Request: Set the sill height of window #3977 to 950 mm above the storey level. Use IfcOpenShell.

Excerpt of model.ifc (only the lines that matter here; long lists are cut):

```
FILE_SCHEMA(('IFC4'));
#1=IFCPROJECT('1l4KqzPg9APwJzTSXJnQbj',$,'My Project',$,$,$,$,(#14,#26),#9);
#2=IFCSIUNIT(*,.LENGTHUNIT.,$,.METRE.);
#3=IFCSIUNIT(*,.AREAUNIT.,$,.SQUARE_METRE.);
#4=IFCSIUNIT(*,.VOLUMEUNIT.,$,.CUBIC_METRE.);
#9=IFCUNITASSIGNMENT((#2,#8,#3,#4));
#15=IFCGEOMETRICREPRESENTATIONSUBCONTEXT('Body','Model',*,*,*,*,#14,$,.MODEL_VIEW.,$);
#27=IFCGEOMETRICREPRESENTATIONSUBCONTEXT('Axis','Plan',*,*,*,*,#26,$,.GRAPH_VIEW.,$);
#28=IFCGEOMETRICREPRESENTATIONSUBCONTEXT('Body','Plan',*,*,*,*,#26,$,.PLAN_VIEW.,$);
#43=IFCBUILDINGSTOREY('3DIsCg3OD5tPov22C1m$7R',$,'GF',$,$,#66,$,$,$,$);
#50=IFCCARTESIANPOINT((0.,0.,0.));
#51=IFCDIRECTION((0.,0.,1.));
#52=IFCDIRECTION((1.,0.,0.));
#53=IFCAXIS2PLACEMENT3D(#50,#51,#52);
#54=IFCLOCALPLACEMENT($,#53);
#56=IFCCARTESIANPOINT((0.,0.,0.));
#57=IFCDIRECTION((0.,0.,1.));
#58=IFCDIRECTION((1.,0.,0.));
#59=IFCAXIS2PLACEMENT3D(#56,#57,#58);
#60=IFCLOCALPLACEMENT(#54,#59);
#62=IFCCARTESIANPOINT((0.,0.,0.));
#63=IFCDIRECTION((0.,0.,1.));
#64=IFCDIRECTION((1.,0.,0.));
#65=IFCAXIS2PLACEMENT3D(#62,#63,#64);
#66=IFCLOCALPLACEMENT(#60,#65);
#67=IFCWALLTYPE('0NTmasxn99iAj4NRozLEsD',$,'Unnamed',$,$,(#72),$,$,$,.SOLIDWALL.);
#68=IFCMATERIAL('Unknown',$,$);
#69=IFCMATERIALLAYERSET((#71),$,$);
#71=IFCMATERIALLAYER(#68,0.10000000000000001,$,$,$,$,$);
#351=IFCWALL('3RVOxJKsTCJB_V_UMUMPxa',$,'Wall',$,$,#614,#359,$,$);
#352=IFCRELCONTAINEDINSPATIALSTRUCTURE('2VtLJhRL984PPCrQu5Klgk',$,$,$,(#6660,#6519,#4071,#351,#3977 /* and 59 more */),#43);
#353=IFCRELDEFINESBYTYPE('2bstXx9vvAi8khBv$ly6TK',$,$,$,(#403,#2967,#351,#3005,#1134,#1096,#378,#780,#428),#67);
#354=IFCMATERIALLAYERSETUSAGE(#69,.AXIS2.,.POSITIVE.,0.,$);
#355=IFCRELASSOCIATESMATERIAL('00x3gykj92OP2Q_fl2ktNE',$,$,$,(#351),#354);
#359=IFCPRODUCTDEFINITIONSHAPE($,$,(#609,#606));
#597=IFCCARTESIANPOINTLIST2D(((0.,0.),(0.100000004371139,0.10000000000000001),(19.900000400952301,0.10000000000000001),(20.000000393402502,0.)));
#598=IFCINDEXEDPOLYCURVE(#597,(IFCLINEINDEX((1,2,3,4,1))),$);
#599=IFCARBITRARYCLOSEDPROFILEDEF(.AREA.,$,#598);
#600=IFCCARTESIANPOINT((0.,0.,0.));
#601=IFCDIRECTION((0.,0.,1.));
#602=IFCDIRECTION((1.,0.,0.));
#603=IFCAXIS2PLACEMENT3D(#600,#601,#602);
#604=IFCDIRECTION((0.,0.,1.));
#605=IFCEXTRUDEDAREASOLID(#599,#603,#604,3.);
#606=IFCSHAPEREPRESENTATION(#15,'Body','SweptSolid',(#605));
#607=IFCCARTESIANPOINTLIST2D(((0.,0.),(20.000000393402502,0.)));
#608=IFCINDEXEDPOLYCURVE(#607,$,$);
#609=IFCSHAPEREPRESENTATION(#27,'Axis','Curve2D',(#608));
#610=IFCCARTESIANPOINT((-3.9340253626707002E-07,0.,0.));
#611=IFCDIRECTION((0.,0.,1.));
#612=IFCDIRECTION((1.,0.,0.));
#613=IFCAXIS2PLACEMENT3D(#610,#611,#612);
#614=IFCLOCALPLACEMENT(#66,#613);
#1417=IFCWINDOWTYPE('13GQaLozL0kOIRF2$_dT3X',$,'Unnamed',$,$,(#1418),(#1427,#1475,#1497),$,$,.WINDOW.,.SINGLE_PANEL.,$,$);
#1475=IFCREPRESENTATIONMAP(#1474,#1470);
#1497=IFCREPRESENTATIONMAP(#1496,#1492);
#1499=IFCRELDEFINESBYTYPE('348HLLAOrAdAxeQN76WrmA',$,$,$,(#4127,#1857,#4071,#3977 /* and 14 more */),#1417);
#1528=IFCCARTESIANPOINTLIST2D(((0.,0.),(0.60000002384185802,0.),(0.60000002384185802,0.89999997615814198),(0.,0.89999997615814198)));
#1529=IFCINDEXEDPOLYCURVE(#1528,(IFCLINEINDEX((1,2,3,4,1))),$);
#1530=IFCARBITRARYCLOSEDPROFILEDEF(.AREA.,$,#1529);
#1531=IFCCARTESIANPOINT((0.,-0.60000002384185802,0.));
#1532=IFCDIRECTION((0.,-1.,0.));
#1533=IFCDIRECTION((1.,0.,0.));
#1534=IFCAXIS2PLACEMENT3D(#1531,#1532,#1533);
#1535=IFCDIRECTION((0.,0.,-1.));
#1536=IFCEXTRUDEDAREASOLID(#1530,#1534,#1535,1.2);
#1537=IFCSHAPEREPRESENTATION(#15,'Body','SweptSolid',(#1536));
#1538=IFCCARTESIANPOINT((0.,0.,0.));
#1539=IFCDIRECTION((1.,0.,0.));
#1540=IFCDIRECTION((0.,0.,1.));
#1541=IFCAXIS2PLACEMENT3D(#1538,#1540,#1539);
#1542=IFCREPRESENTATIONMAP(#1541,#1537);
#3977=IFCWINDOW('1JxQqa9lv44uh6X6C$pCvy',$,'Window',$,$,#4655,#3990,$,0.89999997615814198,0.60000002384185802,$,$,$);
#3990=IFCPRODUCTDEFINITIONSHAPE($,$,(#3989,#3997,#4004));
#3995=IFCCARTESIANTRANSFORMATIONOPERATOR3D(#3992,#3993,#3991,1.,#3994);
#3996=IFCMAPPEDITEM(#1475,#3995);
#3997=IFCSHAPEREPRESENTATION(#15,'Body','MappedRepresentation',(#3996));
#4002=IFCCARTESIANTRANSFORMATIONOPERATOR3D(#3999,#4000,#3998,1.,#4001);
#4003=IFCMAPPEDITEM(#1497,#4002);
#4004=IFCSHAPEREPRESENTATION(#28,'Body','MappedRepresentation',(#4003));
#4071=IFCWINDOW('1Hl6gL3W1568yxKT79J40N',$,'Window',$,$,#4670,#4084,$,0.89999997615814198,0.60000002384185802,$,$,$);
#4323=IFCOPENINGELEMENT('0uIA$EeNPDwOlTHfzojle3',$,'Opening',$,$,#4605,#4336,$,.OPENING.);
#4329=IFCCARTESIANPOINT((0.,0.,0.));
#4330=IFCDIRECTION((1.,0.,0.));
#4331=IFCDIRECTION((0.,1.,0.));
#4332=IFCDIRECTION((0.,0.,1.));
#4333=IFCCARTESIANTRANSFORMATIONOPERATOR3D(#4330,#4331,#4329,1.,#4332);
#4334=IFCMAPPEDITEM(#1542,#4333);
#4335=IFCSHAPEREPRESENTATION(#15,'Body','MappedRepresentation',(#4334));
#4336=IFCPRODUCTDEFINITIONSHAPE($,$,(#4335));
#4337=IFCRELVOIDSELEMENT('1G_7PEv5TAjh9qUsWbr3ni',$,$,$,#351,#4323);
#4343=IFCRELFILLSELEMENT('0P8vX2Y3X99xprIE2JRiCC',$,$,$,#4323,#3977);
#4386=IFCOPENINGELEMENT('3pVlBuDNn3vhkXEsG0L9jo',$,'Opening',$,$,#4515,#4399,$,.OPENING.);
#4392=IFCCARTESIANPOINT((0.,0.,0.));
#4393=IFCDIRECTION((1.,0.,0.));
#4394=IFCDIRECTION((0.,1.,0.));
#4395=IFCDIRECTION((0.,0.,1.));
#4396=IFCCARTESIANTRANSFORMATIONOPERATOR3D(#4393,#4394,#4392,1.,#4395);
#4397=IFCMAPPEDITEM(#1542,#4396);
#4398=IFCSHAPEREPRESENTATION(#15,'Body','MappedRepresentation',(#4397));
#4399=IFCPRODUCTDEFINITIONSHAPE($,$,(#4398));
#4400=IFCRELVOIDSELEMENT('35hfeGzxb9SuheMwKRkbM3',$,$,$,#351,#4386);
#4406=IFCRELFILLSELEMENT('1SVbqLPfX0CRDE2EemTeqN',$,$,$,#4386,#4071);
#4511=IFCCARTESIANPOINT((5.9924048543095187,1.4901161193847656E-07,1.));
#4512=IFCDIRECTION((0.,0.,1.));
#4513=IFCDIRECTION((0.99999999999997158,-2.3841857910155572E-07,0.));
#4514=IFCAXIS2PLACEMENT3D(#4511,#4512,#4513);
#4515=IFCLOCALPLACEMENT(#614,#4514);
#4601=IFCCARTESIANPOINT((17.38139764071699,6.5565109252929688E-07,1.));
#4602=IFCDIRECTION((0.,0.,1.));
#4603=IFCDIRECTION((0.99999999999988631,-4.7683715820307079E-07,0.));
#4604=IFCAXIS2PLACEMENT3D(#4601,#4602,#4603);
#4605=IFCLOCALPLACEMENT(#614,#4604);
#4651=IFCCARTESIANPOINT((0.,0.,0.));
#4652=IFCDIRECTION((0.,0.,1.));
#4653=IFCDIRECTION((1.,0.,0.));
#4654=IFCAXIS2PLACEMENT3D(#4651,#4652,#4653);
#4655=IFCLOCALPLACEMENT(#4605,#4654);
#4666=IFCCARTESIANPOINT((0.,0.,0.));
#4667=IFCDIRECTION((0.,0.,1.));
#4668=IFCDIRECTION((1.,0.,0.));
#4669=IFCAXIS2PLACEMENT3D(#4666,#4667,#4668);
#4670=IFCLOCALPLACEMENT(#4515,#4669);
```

```python
import numpy as np
import ifcopenshell
import ifcopenshell.api.geometry
import ifcopenshell.geom
import ifcopenshell.util.element
import ifcopenshell.util.placement
import ifcopenshell.util.shape
import ifcopenshell.util.unit

model = ifcopenshell.open("model.ifc")
unit_scale = ifcopenshell.util.unit.calculate_unit_scale(model)

window = model.by_guid("1JxQqa9lv44uh6X6C$pCvy")
opening = window.FillsVoids[0].RelatingOpeningElement
storey = ifcopenshell.util.element.get_container(window, ifc_class="IfcBuildingStorey")
level = ifcopenshell.util.placement.get_local_placement(storey.ObjectPlacement)[2, 3]

# The opening's origin need not be at the sill, so measure its lowest point.
shape = ifcopenshell.geom.create_shape(ifcopenshell.geom.settings(), opening)
bottom = ifcopenshell.util.shape.get_shape_bottom_elevation(shape, shape.geometry) / unit_scale
dz = level + 0.95 - bottom

shift = np.array([0.0, 0.0, dz])
# The window is placed relative to its opening, so it follows when the opening moves.
matrix = ifcopenshell.util.placement.get_local_placement(opening.ObjectPlacement)
matrix[:3, 3] += shift
ifcopenshell.api.geometry.edit_object_placement(
    model, product=opening, matrix=matrix, is_si=False, should_transform_children=True
)

print(f"moved by {dz * unit_scale:+.3f} m")

model.write("model_rev.ifc")
```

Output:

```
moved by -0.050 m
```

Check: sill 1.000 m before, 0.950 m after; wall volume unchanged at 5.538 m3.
